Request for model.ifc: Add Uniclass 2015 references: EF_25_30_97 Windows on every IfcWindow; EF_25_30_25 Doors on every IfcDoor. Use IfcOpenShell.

First a look at what the model holds.

```python
import ifcopenshell

model = ifcopenshell.open("model.ifc")
print(model.schema)
print("classifications:", [c.Name for c in model.by_type("IfcClassification")])
for ifc_class in ("IfcDoor", "IfcRoof", "IfcStair", "IfcWall", "IfcWindow"):
    print(ifc_class, len(model.by_type(ifc_class)))
```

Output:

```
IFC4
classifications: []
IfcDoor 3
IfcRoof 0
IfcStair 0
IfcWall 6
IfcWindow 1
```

```python
import ifcopenshell
import ifcopenshell.api.classification

model = ifcopenshell.open("model.ifc")

system = ifcopenshell.api.classification.add_classification(model, classification="Uniclass 2015")

codes = {
    "IfcWindow": ("EF_25_30_97", "Windows"),
    "IfcDoor": ("EF_25_30_25", "Doors"),
}
for ifc_class, (code, name) in codes.items():
    products = model.by_type(ifc_class)
    ifcopenshell.api.classification.add_reference(
        model, products=products, classification=system, identification=code, name=name
    )
    print(code, len(products))

model.write("model-out.ifc")
```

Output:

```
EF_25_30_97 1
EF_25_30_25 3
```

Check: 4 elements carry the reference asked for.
